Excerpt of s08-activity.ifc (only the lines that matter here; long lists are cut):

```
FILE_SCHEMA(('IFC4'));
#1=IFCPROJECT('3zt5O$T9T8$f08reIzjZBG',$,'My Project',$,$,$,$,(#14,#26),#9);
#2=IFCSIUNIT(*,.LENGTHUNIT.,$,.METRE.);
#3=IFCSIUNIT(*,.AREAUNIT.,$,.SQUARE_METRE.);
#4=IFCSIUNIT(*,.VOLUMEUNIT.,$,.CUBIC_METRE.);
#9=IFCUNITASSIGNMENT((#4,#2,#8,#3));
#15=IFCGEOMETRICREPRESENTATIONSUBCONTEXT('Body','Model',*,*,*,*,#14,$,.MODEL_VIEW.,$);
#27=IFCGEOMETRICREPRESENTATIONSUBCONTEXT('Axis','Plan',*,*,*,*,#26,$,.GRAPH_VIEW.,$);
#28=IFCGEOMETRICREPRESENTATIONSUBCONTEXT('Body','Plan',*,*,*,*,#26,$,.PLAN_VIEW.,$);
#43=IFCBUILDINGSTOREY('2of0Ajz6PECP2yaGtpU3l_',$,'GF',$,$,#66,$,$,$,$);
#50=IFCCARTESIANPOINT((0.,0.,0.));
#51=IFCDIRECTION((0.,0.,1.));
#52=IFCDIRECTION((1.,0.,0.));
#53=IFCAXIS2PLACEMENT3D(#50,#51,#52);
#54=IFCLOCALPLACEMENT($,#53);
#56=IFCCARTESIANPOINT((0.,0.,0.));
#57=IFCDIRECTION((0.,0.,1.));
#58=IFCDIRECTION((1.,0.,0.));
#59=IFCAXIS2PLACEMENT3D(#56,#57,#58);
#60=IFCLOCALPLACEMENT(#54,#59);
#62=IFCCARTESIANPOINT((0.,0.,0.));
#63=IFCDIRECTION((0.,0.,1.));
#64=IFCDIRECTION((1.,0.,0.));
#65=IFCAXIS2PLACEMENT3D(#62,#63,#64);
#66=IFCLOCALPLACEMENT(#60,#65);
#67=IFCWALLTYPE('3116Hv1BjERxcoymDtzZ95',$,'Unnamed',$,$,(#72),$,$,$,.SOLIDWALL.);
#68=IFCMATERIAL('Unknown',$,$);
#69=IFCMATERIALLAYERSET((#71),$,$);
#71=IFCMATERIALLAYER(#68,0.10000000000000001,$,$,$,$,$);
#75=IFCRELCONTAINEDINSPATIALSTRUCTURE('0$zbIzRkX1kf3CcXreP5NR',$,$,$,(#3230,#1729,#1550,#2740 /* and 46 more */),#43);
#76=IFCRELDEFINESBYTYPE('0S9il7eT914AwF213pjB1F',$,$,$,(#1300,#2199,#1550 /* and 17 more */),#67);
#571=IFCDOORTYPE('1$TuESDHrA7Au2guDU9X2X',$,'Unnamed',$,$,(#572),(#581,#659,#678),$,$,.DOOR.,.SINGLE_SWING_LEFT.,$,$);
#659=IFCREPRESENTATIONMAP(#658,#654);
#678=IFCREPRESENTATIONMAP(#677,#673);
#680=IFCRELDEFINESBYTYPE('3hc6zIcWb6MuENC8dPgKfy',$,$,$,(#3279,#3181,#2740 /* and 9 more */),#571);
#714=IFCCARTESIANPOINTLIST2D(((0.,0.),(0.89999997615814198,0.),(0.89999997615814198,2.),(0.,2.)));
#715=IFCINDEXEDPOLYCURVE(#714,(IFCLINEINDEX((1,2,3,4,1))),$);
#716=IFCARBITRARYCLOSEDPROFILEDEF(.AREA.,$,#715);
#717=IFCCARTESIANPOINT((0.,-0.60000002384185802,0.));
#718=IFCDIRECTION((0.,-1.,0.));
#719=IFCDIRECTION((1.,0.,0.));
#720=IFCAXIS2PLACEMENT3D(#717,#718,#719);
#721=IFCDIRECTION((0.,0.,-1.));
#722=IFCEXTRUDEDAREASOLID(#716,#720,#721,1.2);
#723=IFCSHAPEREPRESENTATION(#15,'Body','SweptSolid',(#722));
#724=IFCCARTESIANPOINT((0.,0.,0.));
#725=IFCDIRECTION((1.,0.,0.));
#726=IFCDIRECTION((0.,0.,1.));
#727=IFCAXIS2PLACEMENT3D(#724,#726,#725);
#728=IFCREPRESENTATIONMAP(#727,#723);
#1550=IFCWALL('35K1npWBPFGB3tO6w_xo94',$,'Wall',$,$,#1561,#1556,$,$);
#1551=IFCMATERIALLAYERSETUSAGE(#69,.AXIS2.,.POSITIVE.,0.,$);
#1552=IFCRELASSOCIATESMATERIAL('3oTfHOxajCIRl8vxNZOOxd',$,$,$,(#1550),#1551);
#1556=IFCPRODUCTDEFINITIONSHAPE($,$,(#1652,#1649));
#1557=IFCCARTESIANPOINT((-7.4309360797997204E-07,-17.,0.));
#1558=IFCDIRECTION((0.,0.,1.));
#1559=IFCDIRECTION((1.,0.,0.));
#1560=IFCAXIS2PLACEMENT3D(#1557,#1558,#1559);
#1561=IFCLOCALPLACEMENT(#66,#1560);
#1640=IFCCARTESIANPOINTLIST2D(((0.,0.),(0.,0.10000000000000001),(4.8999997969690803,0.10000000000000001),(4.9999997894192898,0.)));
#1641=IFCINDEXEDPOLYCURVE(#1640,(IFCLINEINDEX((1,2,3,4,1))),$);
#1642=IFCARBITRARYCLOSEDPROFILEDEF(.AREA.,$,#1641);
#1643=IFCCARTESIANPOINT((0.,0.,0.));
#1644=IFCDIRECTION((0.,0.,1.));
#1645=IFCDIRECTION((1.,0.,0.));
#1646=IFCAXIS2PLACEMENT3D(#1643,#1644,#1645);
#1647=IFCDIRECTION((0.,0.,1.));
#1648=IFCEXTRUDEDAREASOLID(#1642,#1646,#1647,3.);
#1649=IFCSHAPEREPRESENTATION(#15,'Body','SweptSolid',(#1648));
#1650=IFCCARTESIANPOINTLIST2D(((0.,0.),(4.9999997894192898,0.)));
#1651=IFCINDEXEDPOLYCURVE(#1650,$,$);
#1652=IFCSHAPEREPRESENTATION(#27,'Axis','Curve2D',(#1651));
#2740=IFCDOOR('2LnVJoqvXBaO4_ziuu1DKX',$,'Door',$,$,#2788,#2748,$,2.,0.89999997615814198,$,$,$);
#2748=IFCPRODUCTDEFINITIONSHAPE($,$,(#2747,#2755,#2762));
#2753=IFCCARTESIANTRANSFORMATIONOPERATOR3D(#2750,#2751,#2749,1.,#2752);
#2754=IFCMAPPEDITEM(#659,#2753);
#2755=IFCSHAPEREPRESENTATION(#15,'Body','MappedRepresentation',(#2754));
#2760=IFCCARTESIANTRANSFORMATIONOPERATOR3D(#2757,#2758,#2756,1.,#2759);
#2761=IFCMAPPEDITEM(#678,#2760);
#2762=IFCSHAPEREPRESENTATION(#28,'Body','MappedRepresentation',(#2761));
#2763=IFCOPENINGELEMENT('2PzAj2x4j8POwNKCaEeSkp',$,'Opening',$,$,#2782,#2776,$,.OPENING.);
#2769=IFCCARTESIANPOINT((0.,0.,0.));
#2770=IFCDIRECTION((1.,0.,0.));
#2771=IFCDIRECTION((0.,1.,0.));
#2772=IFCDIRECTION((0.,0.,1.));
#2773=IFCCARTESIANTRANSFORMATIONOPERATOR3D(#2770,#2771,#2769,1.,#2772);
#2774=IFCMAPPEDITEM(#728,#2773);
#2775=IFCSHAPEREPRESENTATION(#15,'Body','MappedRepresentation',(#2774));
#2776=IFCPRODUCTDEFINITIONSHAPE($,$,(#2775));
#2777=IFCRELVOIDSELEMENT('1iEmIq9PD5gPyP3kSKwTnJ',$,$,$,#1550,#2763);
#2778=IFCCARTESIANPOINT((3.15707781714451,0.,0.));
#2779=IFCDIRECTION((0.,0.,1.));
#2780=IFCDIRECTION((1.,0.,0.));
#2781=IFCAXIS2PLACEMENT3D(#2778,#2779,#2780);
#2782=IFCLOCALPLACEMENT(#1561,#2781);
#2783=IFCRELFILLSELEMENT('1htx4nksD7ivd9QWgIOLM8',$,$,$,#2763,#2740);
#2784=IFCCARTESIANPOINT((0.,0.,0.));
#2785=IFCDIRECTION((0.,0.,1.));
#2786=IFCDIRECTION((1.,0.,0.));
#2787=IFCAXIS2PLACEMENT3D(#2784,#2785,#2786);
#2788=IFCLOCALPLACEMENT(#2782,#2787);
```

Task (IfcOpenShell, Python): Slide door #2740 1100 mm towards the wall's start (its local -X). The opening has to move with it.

```python
import ifcopenshell
import ifcopenshell.api.geometry
import ifcopenshell.util.placement
import ifcopenshell.util.unit

model = ifcopenshell.open("s08-activity.ifc")
unit_scale = ifcopenshell.util.unit.calculate_unit_scale(model)

door = model.by_guid("2LnVJoqvXBaO4_ziuu1DKX")
opening = door.FillsVoids[0].RelatingOpeningElement
wall = opening.VoidsElements[0].RelatingBuildingElement

wall_matrix = ifcopenshell.util.placement.get_local_placement(wall.ObjectPlacement)
shift = wall_matrix[:3, 0] * -1.1 / unit_scale
before = ifcopenshell.util.placement.get_local_placement(door.ObjectPlacement)[:3, 3].copy()

# The door is placed relative to its opening, so it follows when the opening moves.
matrix = ifcopenshell.util.placement.get_local_placement(opening.ObjectPlacement)
matrix[:3, 3] += shift
ifcopenshell.api.geometry.edit_object_placement(
    model, product=opening, matrix=matrix, is_si=False, should_transform_children=True
)

after = ifcopenshell.util.placement.get_local_placement(door.ObjectPlacement)[:3, 3]
print("door moved by", (after - before).round(3) + 0.0)

model.write("s08-activity-out.ifc")
```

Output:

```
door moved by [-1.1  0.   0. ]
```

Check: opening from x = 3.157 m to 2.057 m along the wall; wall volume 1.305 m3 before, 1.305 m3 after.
